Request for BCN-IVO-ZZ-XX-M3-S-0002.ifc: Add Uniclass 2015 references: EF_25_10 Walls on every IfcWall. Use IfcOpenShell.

First a look at what the model holds.

```python
import ifcopenshell

model = ifcopenshell.open("BCN-IVO-ZZ-XX-M3-S-0002.ifc")
print(model.schema)
print("classifications:", [c.Name for c in model.by_type("IfcClassification")])
for ifc_class in ("IfcDoor", "IfcRoof", "IfcStair", "IfcWall", "IfcWindow"):
    print(ifc_class, len(model.by_type(ifc_class)))
```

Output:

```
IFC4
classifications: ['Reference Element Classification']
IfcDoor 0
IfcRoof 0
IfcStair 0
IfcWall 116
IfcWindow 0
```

```python
import ifcopenshell
import ifcopenshell.api.classification

model = ifcopenshell.open("BCN-IVO-ZZ-XX-M3-S-0002.ifc")

system = ifcopenshell.api.classification.add_classification(model, classification="Uniclass 2015")

codes = {
    "IfcWall": ("EF_25_10", "Walls"),
}
for ifc_class, (code, name) in codes.items():
    products = model.by_type(ifc_class)
    ifcopenshell.api.classification.add_reference(
        model, products=products, classification=system, identification=code, name=name
    )
    print(code, len(products))

model.write("BCN-IVO-ZZ-XX-M3-S-0002_edited.ifc")
```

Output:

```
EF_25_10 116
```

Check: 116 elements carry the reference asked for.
